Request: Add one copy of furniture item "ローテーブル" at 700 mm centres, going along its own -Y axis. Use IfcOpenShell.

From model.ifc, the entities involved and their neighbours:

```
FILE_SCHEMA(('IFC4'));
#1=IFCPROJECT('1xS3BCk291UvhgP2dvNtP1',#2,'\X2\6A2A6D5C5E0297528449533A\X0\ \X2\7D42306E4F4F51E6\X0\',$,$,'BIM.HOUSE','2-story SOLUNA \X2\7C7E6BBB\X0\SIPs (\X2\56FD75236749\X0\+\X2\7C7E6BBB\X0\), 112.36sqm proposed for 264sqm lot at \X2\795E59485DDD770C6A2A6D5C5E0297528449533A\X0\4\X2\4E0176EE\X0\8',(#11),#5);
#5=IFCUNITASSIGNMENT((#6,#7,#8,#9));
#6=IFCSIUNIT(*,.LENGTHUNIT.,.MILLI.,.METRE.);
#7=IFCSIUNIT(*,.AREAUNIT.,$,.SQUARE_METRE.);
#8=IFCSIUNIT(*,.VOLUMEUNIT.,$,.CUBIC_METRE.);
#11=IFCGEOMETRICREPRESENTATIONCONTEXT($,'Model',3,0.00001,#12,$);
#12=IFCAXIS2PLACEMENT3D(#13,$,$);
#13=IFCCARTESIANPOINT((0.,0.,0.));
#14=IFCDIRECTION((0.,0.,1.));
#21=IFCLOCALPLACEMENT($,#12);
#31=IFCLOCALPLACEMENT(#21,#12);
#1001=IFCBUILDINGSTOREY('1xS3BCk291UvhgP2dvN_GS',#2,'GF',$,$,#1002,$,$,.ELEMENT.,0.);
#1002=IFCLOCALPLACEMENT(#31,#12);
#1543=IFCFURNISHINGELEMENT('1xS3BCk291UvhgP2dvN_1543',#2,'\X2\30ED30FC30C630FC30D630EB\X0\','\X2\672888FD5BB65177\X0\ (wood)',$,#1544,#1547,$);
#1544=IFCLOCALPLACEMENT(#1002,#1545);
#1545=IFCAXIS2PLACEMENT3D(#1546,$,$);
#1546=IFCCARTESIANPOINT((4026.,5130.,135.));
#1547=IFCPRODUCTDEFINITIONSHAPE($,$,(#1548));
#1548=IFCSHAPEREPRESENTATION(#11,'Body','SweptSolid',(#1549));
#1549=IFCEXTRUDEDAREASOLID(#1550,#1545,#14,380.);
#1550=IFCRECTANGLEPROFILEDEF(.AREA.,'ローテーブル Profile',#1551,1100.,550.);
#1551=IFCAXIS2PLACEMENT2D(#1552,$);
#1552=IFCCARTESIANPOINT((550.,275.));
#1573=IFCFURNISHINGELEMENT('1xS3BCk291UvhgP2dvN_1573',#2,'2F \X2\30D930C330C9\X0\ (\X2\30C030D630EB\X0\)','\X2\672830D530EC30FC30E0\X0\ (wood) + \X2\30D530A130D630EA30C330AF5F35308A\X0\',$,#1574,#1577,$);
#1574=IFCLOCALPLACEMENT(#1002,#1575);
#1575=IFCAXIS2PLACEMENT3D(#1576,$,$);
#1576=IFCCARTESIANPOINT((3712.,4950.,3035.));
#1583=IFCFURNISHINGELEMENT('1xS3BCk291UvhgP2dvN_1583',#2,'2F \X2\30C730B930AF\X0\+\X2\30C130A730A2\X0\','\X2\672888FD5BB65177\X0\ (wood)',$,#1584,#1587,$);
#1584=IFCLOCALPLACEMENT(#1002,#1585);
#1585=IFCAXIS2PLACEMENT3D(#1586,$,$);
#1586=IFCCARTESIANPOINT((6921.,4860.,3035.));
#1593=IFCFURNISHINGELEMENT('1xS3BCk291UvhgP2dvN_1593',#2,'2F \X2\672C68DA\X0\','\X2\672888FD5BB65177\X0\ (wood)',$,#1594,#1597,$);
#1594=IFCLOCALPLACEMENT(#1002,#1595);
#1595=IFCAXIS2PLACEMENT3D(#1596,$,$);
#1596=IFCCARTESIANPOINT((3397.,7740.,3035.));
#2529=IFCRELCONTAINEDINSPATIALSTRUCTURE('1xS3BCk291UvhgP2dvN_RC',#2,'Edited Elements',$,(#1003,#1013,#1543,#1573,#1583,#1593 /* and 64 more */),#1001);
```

```python
import ifcopenshell
import ifcopenshell.api.geometry
import ifcopenshell.api.root
import ifcopenshell.util.element
import ifcopenshell.util.placement
import ifcopenshell.util.unit

model = ifcopenshell.open("model.ifc")
unit_scale = ifcopenshell.util.unit.calculate_unit_scale(model)


def reuse_history(source, copy):
    """copy_class also copies each property set's owner history, people and application; keep the originals."""
    for rel in copy.IsDefinedBy:
        if rel.is_a("IfcRelDefinesByProperties") and (history := rel.RelatingPropertyDefinition.OwnerHistory):
            rel.RelatingPropertyDefinition.OwnerHistory = source.OwnerHistory
            ifcopenshell.util.element.remove_deep2(model, history)


source = model.by_id(1543)
base = ifcopenshell.util.placement.get_local_placement(source.ObjectPlacement)
step = -base[:3, 1] * 0.7 / unit_scale

for i in range(1, 2):
    copy = ifcopenshell.api.root.copy_class(model, product=source)
    copy.Representation = ifcopenshell.util.element.copy_deep(
        model, source.Representation, exclude=["IfcGeometricRepresentationContext", "IfcRepresentationMap"]
    )
    reuse_history(source, copy)
    matrix = base.copy()
    matrix[:3, 3] += i * step
    print("added at", matrix[:3, 3].round(3) + 0.0)
    ifcopenshell.api.geometry.edit_object_placement(model, product=copy, matrix=matrix, is_si=False)

model.write("model_edited.ifc")
```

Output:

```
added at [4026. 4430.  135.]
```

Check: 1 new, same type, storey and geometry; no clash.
